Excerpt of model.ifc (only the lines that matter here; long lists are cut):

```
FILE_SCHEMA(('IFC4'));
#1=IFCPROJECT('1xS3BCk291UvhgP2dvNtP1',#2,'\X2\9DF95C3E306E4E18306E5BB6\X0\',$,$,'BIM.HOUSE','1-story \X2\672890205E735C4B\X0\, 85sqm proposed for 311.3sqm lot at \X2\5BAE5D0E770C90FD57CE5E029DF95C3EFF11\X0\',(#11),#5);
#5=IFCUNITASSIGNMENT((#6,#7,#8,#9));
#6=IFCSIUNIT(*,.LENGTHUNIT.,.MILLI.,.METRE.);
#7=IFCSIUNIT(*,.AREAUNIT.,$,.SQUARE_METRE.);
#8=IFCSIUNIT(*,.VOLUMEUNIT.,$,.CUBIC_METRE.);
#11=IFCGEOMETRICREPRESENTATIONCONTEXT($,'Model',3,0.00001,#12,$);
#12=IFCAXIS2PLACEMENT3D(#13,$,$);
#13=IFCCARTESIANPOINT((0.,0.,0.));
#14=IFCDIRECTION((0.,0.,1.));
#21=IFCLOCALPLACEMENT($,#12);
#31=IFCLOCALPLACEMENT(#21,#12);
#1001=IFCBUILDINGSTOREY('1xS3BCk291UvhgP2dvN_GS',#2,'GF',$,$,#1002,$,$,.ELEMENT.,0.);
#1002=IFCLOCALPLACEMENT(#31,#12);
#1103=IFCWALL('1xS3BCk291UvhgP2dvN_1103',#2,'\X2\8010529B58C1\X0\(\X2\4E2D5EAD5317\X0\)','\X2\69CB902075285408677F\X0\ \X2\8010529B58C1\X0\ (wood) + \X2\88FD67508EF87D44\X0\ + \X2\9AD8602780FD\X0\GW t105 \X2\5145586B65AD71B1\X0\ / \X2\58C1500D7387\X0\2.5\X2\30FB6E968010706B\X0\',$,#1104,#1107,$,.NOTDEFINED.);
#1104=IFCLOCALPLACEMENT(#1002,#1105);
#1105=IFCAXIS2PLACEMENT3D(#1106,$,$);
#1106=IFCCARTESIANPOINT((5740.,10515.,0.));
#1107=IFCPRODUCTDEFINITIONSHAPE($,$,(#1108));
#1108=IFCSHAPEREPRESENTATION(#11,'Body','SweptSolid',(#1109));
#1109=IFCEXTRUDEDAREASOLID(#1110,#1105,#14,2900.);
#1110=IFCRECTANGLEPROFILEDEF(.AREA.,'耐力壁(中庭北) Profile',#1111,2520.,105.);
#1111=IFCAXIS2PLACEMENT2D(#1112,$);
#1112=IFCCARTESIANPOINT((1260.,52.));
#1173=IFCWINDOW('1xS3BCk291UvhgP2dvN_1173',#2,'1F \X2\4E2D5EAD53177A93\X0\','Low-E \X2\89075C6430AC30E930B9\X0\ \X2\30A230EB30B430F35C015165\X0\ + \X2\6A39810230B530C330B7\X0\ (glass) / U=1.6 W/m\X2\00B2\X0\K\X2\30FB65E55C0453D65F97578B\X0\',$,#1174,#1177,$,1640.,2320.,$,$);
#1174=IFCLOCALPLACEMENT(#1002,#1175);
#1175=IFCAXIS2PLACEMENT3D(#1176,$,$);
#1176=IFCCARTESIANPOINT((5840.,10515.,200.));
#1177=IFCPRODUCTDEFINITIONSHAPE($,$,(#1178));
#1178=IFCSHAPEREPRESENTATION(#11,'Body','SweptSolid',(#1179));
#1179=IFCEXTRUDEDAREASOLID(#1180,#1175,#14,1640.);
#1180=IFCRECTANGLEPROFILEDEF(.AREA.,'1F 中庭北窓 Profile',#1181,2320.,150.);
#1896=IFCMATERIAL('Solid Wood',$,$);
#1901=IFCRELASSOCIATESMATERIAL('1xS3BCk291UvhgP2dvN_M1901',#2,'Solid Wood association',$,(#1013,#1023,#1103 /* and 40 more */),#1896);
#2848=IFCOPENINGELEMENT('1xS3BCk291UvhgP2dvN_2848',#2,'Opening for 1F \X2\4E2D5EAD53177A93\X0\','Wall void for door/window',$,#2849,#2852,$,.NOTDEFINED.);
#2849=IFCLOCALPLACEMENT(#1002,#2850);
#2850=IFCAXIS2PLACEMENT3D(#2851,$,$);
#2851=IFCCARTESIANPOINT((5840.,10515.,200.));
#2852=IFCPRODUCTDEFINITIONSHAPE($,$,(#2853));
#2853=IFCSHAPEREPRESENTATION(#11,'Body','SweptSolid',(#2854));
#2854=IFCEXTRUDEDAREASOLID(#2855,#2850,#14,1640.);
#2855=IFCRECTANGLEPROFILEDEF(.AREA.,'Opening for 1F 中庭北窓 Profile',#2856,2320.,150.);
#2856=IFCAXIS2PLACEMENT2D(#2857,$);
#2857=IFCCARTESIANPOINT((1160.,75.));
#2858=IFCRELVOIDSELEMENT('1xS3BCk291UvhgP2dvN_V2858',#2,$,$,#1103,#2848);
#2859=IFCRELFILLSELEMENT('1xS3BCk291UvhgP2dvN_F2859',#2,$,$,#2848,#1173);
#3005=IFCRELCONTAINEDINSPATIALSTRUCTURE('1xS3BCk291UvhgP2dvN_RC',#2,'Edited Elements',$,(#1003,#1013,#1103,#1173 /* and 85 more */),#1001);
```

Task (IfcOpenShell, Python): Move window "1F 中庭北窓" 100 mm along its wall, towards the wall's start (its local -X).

```python
import ifcopenshell
import ifcopenshell.api.geometry
import ifcopenshell.util.placement

model = ifcopenshell.open("model.ifc")

window = model.by_id(1173)
opening = window.FillsVoids[0].RelatingOpeningElement
wall = opening.VoidsElements[0].RelatingBuildingElement

wall_matrix = ifcopenshell.util.placement.get_local_placement(wall.ObjectPlacement)
shift = wall_matrix[:3, 0] * -100.0
before = ifcopenshell.util.placement.get_local_placement(window.ObjectPlacement)[:3, 3].copy()

# The window is not placed relative to its opening, so move both.
for product in (opening, window):
    matrix = ifcopenshell.util.placement.get_local_placement(product.ObjectPlacement)
    matrix[:3, 3] += shift
    ifcopenshell.api.geometry.edit_object_placement(model, product=product, matrix=matrix, is_si=False)

after = ifcopenshell.util.placement.get_local_placement(window.ObjectPlacement)[:3, 3]
print("window moved by", (after - before).round(3) + 0.0)

model.write("model_v2.ifc")
```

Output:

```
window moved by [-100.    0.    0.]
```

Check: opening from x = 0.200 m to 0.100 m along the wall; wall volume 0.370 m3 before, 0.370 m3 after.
